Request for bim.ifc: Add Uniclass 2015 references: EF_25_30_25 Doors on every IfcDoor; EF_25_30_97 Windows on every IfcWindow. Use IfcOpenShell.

First a look at what the model holds.

```python
import ifcopenshell

model = ifcopenshell.open("bim.ifc")
print(model.schema)
print("classifications:", [c.Name for c in model.by_type("IfcClassification")])
for ifc_class in ("IfcDoor", "IfcRoof", "IfcStair", "IfcWall", "IfcWindow"):
    print(ifc_class, len(model.by_type(ifc_class)))
```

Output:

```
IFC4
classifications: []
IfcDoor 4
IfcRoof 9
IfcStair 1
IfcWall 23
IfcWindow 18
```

```python
import ifcopenshell
import ifcopenshell.api.classification

model = ifcopenshell.open("bim.ifc")

system = ifcopenshell.api.classification.add_classification(model, classification="Uniclass 2015")

codes = {
    "IfcDoor": ("EF_25_30_25", "Doors"),
    "IfcWindow": ("EF_25_30_97", "Windows"),
}
for ifc_class, (code, name) in codes.items():
    products = model.by_type(ifc_class)
    ifcopenshell.api.classification.add_reference(
        model, products=products, classification=system, identification=code, name=name
    )
    print(code, len(products))

model.write("bim_v2.ifc")
```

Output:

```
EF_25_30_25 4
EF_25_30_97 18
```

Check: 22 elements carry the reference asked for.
